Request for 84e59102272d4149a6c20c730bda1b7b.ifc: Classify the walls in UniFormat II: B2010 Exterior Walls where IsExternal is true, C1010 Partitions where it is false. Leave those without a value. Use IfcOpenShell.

First a look at what the model holds.

```python
import ifcopenshell
import ifcopenshell.util.element

model = ifcopenshell.open("84e59102272d4149a6c20c730bda1b7b.ifc")
print(model.schema)
print("classifications:", [c.Name for c in model.by_type("IfcClassification")])
values = [ifcopenshell.util.element.get_pset(e, "Pset_WallCommon", "IsExternal") for e in model.by_type("IfcWall")]
for value in (True, False, None):
    print("IsExternal", value, values.count(value))
```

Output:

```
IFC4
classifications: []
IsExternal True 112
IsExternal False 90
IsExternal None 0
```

```python
import ifcopenshell
import ifcopenshell.api.classification
import ifcopenshell.util.element

model = ifcopenshell.open("84e59102272d4149a6c20c730bda1b7b.ifc")

system = ifcopenshell.api.classification.add_classification(model, classification="UniFormat II")

walls = model.by_type("IfcWall")
external = {e: ifcopenshell.util.element.get_pset(e, "Pset_WallCommon", "IsExternal") for e in walls}
for flag, code, name in ((True, "B2010", "Exterior Walls"), (False, "C1010", "Partitions")):
    products = [e for e in walls if external[e] is flag]
    ifcopenshell.api.classification.add_reference(
        model, products=products, classification=system, identification=code, name=name
    )
    print(code, len(products))

model.write("84e59102272d4149a6c20c730bda1b7b_v2.ifc")
```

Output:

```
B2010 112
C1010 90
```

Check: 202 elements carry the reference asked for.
